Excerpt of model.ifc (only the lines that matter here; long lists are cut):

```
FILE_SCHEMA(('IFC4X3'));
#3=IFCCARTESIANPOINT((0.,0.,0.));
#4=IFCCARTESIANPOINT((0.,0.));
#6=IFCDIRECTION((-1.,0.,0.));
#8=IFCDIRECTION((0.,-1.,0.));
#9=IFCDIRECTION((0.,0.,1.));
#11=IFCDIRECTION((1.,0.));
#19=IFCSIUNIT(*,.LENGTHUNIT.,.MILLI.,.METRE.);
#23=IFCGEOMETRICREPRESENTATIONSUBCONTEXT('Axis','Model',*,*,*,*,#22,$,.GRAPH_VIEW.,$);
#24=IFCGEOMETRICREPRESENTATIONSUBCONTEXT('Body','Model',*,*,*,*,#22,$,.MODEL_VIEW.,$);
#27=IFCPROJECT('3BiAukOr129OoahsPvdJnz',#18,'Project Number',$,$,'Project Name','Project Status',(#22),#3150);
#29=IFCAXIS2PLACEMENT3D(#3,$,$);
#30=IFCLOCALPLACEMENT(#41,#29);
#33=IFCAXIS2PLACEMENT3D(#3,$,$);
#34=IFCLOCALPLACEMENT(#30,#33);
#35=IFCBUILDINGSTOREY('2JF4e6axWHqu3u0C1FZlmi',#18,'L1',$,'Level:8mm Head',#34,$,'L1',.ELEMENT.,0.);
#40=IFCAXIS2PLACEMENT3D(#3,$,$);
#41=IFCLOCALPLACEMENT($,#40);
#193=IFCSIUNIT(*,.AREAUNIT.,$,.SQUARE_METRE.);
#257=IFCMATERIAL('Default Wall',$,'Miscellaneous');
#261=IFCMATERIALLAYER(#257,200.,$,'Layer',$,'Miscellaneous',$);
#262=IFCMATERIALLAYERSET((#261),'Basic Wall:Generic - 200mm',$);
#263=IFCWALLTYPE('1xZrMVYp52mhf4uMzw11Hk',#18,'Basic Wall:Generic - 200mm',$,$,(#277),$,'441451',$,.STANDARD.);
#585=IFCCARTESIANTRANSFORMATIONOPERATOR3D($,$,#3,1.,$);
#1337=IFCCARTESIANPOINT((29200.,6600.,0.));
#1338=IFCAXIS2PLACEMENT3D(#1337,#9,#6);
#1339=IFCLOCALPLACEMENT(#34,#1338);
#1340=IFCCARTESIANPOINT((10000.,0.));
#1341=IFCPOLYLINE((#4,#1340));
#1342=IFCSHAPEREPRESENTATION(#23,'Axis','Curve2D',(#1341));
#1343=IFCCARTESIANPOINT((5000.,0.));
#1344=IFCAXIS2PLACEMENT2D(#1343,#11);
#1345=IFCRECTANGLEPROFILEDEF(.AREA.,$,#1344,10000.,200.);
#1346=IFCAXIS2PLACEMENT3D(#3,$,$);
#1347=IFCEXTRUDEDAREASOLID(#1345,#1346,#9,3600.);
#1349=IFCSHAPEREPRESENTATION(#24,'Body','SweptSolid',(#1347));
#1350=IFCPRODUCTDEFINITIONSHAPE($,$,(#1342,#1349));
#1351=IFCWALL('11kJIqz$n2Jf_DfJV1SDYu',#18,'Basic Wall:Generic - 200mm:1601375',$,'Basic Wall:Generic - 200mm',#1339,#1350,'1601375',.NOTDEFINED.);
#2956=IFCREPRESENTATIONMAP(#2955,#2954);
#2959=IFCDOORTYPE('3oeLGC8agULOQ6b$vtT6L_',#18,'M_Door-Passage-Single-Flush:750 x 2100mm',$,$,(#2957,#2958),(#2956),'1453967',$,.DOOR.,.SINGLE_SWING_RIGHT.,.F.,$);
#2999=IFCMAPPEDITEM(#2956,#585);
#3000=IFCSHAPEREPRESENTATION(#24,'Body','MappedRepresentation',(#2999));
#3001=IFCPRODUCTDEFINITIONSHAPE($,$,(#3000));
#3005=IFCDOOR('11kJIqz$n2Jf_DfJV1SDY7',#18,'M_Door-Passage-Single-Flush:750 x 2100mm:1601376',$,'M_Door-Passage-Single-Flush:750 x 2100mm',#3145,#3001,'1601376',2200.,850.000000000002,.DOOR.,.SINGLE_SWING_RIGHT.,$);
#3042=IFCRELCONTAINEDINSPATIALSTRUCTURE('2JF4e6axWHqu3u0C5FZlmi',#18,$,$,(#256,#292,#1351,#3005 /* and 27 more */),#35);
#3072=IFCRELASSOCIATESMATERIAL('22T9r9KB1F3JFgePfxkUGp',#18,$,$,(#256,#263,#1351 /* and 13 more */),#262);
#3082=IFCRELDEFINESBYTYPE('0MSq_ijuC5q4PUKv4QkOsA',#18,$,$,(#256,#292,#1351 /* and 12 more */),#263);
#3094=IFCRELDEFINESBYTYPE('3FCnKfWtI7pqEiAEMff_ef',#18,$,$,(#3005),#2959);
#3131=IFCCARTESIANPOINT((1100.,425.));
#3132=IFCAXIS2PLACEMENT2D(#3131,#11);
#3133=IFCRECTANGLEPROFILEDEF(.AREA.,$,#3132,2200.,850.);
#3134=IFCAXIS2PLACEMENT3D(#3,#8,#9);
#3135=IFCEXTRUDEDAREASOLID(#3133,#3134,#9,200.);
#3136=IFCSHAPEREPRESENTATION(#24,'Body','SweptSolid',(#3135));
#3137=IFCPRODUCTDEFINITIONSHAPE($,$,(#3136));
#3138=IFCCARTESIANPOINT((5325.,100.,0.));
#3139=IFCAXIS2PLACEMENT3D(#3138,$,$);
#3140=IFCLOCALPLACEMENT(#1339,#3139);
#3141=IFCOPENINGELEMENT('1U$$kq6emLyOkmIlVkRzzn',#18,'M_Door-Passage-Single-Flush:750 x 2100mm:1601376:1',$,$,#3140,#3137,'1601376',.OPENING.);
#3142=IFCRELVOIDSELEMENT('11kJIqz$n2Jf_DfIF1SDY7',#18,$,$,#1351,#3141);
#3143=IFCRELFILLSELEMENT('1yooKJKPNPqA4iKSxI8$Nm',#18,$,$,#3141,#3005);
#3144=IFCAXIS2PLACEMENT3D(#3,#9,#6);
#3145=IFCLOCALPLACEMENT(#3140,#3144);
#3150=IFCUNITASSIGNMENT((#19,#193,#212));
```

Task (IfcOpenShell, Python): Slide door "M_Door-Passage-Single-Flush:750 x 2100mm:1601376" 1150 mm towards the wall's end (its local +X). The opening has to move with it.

```python
import ifcopenshell
import ifcopenshell.api.geometry
import ifcopenshell.util.placement

model = ifcopenshell.open("model.ifc")

door = model.by_guid("11kJIqz$n2Jf_DfJV1SDY7")
opening = door.FillsVoids[0].RelatingOpeningElement
wall = opening.VoidsElements[0].RelatingBuildingElement

wall_matrix = ifcopenshell.util.placement.get_local_placement(wall.ObjectPlacement)
shift = wall_matrix[:3, 0] * 1150.0
before = ifcopenshell.util.placement.get_local_placement(door.ObjectPlacement)[:3, 3].copy()

# The door is placed relative to its opening, so it follows when the opening moves.
matrix = ifcopenshell.util.placement.get_local_placement(opening.ObjectPlacement)
matrix[:3, 3] += shift
ifcopenshell.api.geometry.edit_object_placement(
    model, product=opening, matrix=matrix, is_si=False, should_transform_children=True
)

after = ifcopenshell.util.placement.get_local_placement(door.ObjectPlacement)[:3, 3]
print("door moved by", (after - before).round(3) + 0.0)

model.write("model_rev.ifc")
```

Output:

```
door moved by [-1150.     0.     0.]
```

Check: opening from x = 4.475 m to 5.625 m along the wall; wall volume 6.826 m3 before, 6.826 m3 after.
